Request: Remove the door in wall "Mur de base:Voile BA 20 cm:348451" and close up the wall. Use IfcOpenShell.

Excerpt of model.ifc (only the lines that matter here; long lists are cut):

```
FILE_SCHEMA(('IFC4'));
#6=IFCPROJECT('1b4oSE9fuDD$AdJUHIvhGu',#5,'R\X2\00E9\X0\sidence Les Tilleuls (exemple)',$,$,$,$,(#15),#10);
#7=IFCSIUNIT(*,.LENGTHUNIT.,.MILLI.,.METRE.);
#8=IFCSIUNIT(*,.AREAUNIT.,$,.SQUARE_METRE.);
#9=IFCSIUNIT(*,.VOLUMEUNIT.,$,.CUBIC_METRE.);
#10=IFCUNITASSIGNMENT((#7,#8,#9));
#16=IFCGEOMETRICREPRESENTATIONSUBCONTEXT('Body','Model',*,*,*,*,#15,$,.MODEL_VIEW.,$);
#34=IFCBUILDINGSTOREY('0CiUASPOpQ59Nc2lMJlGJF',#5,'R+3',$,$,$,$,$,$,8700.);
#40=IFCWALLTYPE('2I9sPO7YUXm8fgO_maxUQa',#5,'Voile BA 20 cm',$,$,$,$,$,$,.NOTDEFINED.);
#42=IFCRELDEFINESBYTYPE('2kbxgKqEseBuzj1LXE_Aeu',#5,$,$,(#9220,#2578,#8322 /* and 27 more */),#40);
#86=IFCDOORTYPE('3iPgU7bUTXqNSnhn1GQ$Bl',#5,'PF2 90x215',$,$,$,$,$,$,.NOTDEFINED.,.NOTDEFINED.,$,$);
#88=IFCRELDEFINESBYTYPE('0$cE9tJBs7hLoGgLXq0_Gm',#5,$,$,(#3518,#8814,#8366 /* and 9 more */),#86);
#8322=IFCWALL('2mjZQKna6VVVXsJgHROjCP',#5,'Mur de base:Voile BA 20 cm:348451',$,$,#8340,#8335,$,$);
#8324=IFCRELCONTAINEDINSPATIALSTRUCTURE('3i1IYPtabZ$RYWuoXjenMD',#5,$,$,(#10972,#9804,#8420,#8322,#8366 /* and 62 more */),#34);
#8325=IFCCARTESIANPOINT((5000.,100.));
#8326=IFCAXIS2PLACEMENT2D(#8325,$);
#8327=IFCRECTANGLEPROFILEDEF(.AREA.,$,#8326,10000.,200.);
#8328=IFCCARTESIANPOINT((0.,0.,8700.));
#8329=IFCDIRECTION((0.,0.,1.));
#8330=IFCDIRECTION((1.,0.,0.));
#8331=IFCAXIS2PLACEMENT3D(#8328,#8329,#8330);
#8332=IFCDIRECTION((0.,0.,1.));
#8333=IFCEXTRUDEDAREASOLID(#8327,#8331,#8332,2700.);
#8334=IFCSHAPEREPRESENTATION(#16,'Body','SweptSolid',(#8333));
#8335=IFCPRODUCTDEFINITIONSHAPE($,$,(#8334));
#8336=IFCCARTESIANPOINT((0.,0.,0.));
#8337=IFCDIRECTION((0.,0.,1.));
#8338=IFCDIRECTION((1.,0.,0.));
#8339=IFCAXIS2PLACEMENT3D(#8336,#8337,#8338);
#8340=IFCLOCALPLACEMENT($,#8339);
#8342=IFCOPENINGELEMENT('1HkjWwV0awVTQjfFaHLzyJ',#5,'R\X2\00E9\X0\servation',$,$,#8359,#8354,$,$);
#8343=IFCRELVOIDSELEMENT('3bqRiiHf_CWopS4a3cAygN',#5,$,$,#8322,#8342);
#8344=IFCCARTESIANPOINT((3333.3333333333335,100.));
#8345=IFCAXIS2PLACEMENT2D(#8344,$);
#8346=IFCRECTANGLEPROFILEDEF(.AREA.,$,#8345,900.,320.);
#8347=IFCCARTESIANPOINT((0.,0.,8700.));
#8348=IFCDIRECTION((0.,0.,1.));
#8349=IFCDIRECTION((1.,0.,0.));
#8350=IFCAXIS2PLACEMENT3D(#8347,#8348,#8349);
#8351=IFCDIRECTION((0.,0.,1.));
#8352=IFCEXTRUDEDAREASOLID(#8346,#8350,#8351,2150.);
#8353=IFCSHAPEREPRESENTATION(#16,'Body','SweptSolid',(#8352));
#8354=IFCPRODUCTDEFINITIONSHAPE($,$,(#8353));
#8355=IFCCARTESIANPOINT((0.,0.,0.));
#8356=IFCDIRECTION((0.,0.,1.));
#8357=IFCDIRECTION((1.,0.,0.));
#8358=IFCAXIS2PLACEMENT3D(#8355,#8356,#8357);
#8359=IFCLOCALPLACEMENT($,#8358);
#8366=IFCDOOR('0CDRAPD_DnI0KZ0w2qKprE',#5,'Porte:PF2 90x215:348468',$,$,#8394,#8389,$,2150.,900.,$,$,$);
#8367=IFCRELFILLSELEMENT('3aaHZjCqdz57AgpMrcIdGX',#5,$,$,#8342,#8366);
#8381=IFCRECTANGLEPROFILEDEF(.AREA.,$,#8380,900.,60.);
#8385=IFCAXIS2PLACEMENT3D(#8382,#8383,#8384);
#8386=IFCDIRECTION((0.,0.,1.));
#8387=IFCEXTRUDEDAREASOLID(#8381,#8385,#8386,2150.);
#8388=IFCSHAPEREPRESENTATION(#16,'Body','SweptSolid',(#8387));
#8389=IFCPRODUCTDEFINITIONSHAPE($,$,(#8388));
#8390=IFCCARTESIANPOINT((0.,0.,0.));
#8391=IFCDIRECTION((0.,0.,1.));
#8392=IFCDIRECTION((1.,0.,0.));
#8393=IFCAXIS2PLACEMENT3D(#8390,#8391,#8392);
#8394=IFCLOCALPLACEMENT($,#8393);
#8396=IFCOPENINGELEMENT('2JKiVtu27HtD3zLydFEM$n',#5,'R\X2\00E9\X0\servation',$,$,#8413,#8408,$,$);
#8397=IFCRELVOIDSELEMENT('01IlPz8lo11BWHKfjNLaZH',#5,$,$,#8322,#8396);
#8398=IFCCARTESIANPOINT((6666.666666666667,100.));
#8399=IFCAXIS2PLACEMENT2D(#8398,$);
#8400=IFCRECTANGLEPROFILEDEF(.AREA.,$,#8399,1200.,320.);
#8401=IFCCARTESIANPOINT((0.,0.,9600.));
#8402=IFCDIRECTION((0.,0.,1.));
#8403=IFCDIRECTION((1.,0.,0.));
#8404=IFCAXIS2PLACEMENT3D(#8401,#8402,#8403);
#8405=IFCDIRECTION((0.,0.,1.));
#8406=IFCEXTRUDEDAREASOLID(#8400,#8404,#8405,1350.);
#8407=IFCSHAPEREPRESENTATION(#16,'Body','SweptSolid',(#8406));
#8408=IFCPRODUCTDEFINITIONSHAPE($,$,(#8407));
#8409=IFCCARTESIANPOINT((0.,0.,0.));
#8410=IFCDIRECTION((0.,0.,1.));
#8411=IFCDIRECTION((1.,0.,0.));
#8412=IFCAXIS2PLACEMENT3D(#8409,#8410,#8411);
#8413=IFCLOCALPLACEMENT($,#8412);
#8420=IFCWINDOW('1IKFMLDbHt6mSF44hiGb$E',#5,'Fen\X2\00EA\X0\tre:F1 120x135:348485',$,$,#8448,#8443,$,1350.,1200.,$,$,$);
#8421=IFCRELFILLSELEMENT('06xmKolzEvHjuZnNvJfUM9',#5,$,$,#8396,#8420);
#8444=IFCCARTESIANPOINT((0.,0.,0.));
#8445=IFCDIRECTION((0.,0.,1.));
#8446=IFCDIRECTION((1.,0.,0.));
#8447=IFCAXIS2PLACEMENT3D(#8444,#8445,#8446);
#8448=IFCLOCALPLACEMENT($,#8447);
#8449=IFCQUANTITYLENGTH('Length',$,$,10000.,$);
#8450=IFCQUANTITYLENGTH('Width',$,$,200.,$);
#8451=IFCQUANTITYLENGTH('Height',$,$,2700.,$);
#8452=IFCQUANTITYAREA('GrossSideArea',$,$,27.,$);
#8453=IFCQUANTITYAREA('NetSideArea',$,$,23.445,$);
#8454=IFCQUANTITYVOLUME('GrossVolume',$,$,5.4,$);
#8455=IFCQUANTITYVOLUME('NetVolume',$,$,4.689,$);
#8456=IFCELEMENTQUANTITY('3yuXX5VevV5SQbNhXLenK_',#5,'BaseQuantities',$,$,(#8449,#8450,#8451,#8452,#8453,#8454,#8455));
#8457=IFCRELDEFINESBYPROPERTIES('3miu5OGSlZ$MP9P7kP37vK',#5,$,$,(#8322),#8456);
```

```python
import ifcopenshell
import ifcopenshell.api.feature
import ifcopenshell.api.pset
import ifcopenshell.api.root
import ifcopenshell.geom
import ifcopenshell.util.element
import ifcopenshell.util.shape
import ifcopenshell.util.unit

model = ifcopenshell.open("model.ifc")
area_scale = ifcopenshell.util.unit.calculate_unit_scale(model, "AREAUNIT")
volume_scale = ifcopenshell.util.unit.calculate_unit_scale(model, "VOLUMEUNIT")
settings = ifcopenshell.geom.settings()


def volume(element):
    """Net volume in cubic metres, openings subtracted."""
    shape = ifcopenshell.geom.create_shape(settings, element)
    return ifcopenshell.util.shape.get_volume(shape.geometry)


door = model.by_id(8366)
opening = door.FillsVoids[0].RelatingOpeningElement
wall = opening.VoidsElements[0].RelatingBuildingElement
before = volume(wall)

ifcopenshell.api.root.remove_product(model, product=door)
ifcopenshell.api.feature.remove_feature(model, feature=opening)

after = volume(wall)
thickness = 0.2  # wall thickness in metres

# Update the wall's stored quantities.
qto = model.by_id(ifcopenshell.util.element.get_pset(wall, "BaseQuantities", should_inherit=False)["id"])
ifcopenshell.api.pset.edit_qto(model, qto=qto, properties={
    "NetSideArea": after / thickness / area_scale,
    "NetVolume": after / volume_scale,
})

print(f"wall volume {before:.3f} -> {after:.3f} m3")

model.write("model-out.ifc")
```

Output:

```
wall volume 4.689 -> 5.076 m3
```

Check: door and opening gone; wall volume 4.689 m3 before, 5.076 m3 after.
